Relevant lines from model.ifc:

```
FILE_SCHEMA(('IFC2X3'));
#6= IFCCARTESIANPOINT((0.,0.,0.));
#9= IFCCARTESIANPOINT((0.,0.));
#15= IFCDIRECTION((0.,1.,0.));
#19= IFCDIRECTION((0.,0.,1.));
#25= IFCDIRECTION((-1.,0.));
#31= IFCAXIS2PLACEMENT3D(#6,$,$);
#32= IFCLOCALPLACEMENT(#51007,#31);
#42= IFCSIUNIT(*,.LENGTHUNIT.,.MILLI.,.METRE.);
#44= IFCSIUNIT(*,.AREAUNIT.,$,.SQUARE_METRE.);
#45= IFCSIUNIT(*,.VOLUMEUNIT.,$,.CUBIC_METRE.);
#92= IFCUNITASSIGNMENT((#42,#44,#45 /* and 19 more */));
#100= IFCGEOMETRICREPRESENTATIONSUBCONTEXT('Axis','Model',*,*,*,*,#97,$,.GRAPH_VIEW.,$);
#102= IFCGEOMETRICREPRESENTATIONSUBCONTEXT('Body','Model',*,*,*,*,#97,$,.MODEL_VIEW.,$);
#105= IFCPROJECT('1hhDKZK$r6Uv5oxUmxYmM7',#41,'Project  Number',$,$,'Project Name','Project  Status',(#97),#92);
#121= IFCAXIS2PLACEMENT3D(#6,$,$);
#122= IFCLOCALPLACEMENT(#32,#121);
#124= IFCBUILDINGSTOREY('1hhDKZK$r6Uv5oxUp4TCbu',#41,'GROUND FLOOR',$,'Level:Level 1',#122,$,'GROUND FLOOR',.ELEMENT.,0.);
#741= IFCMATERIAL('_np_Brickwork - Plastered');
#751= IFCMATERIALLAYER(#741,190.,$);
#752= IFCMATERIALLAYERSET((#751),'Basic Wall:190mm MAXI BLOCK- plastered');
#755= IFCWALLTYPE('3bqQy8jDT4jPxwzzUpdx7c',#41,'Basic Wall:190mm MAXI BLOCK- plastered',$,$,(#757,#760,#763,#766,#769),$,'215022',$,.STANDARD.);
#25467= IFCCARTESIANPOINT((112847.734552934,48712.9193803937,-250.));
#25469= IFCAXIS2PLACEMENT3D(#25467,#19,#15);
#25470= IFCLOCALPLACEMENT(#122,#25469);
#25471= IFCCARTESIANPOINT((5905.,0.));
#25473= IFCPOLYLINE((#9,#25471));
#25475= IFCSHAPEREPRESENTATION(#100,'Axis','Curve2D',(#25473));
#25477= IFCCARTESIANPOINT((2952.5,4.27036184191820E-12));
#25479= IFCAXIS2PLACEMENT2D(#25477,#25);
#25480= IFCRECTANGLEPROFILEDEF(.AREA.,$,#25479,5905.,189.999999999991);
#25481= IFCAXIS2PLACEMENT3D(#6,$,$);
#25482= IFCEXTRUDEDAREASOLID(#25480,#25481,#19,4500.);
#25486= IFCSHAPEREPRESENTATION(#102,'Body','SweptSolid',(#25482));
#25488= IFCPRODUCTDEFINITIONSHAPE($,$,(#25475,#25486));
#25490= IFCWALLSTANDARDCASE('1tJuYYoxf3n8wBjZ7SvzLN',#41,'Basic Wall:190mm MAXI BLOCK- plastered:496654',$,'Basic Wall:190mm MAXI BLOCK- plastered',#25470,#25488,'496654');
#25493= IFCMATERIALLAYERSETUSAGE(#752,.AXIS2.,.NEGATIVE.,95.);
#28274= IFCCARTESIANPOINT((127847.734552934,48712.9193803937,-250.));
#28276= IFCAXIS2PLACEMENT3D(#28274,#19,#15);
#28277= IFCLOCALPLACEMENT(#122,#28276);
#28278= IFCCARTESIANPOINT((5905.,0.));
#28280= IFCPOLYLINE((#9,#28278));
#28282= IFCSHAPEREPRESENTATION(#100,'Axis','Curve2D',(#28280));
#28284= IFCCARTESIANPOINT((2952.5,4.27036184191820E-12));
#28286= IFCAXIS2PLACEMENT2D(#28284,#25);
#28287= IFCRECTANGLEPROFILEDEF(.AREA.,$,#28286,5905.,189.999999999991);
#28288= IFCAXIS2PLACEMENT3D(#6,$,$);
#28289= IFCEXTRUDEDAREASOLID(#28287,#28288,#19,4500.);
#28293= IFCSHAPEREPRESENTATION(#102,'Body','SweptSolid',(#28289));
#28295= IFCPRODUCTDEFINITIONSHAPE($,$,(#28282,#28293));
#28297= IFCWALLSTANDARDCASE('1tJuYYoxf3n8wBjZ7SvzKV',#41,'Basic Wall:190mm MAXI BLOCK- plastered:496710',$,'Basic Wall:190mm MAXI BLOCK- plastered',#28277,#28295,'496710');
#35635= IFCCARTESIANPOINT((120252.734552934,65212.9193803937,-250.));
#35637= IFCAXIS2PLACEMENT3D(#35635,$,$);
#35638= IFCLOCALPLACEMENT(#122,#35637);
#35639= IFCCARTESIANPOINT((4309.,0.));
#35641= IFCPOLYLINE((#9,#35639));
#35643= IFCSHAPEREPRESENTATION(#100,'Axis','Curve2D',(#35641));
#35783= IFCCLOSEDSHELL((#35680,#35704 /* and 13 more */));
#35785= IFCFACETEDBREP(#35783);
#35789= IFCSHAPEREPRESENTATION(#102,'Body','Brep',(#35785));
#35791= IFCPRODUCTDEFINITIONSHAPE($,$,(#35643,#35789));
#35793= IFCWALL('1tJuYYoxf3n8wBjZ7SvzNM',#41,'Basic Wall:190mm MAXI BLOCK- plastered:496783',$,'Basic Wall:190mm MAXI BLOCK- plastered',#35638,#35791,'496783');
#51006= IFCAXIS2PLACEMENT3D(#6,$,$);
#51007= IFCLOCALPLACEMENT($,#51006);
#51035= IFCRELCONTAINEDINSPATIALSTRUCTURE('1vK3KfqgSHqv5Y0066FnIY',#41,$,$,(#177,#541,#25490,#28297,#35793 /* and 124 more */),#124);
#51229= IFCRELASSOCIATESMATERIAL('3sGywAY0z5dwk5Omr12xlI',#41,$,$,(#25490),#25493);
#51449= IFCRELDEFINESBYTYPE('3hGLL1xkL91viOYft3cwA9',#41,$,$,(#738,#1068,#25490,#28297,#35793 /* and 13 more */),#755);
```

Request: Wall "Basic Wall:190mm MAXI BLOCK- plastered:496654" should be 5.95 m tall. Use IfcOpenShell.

```python
import ifcopenshell
import ifcopenshell.geom
import ifcopenshell.util.representation
import ifcopenshell.util.shape

model = ifcopenshell.open("model.ifc")
settings = ifcopenshell.geom.settings()


def volume(element):
    """Net volume in cubic metres, openings subtracted."""
    shape = ifcopenshell.geom.create_shape(settings, element)
    return ifcopenshell.util.shape.get_volume(shape.geometry)


wall = model.by_guid("1tJuYYoxf3n8wBjZ7SvzLN")
before = volume(wall)

body = ifcopenshell.util.representation.get_representation(wall, "Model", "Body")
solid = body.Items[0]
old_height = solid.Depth
solid.Depth = 5950.0
after = volume(wall)

print(f"height {old_height:g} -> {solid.Depth:g}, volume {before:.3f} -> {after:.3f} m3")

model.write("model_edited.ifc")
```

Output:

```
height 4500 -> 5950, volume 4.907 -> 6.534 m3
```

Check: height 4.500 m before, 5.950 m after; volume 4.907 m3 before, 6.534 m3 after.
